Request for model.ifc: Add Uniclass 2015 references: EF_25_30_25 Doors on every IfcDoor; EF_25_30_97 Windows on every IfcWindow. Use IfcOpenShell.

First a look at what the model holds.

```python
import ifcopenshell

model = ifcopenshell.open("model.ifc")
print(model.schema)
print("classifications:", [c.Name for c in model.by_type("IfcClassification")])
for ifc_class in ("IfcDoor", "IfcRoof", "IfcStair", "IfcWall", "IfcWindow"):
    print(ifc_class, len(model.by_type(ifc_class)))
```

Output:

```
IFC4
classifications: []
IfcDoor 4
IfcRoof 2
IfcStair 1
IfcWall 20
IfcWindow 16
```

```python
import ifcopenshell
import ifcopenshell.api.classification

model = ifcopenshell.open("model.ifc")

system = ifcopenshell.api.classification.add_classification(model, classification="Uniclass 2015")

codes = {
    "IfcDoor": ("EF_25_30_25", "Doors"),
    "IfcWindow": ("EF_25_30_97", "Windows"),
}
for ifc_class, (code, name) in codes.items():
    products = model.by_type(ifc_class)
    ifcopenshell.api.classification.add_reference(
        model, products=products, classification=system, identification=code, name=name
    )
    print(code, len(products))

model.write("model-out.ifc")
```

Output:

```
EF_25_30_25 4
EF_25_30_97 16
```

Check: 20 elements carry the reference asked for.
